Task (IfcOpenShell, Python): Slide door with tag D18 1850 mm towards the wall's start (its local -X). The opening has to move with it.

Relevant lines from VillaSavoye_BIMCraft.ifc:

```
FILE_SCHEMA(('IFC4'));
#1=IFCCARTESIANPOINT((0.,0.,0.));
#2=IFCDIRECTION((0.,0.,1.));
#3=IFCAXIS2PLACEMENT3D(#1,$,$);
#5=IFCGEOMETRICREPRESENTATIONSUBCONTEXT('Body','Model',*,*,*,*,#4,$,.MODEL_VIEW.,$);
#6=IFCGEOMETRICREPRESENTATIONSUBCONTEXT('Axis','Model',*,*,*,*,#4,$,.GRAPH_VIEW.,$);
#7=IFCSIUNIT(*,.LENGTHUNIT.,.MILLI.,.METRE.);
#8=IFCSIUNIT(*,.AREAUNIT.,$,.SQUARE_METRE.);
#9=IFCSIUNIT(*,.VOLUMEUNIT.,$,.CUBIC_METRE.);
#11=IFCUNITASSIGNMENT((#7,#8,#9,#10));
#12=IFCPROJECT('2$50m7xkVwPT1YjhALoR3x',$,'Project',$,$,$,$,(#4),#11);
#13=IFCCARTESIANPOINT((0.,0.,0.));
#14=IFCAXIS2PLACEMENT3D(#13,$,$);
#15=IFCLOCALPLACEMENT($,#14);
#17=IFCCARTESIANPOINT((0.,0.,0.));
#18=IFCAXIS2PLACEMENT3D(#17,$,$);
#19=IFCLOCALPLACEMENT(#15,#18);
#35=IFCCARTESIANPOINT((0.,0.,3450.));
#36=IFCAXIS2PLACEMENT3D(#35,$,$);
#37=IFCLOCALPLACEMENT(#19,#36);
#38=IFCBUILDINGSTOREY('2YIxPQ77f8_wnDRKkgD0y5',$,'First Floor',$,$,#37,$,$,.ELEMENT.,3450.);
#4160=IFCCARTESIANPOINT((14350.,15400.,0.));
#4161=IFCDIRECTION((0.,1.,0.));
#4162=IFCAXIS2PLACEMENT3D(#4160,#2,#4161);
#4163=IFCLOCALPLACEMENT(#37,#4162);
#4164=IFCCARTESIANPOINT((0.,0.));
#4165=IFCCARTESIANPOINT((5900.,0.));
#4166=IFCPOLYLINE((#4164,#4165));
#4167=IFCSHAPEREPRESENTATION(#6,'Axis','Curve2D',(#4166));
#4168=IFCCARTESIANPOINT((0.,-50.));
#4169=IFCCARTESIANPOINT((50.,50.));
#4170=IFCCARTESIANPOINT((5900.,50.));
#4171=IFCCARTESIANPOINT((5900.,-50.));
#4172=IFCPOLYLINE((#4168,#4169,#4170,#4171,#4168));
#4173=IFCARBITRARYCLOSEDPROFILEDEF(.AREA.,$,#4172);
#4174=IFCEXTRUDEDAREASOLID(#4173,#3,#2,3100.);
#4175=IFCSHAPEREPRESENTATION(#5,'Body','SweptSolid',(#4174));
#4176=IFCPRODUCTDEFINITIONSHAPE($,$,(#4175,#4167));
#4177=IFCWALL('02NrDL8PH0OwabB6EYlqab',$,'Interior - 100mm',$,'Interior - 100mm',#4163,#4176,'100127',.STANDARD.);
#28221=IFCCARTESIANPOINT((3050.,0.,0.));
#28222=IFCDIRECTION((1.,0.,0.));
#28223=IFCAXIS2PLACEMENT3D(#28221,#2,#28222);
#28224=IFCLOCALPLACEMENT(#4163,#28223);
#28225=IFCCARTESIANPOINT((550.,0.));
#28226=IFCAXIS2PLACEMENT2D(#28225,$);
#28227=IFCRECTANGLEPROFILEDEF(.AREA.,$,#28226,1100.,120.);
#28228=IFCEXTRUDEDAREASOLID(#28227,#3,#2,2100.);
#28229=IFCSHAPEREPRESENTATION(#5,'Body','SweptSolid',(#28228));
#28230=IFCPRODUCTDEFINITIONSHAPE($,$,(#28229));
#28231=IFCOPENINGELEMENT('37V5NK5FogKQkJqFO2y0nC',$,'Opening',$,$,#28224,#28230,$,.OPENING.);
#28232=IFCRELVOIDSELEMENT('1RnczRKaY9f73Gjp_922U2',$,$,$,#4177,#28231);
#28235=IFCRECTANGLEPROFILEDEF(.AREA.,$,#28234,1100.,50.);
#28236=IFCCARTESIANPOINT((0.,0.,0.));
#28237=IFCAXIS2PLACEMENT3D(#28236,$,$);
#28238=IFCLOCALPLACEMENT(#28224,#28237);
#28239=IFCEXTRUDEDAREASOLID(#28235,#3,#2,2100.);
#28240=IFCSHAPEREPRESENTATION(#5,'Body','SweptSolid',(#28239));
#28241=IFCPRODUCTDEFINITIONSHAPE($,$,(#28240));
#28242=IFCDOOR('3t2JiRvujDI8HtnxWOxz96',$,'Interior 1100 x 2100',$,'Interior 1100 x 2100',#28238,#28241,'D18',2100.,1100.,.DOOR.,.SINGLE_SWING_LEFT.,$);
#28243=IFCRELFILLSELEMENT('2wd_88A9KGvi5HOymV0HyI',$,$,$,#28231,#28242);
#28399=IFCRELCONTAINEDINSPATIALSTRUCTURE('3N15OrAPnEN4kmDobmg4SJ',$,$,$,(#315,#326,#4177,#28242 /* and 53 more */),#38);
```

```python
import ifcopenshell
import ifcopenshell.api.geometry
import ifcopenshell.util.placement

model = ifcopenshell.open("VillaSavoye_BIMCraft.ifc")

door = model.by_guid("3t2JiRvujDI8HtnxWOxz96")
opening = door.FillsVoids[0].RelatingOpeningElement
wall = opening.VoidsElements[0].RelatingBuildingElement

wall_matrix = ifcopenshell.util.placement.get_local_placement(wall.ObjectPlacement)
shift = wall_matrix[:3, 0] * -1850.0
before = ifcopenshell.util.placement.get_local_placement(door.ObjectPlacement)[:3, 3].copy()

# The door is placed relative to its opening, so it follows when the opening moves.
matrix = ifcopenshell.util.placement.get_local_placement(opening.ObjectPlacement)
matrix[:3, 3] += shift
ifcopenshell.api.geometry.edit_object_placement(
    model, product=opening, matrix=matrix, is_si=False, should_transform_children=True
)

after = ifcopenshell.util.placement.get_local_placement(door.ObjectPlacement)[:3, 3]
print("door moved by", (after - before).round(3) + 0.0)

model.write("VillaSavoye_BIMCraft_v2.ifc")
```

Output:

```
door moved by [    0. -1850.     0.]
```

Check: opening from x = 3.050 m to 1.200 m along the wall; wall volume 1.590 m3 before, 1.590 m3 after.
